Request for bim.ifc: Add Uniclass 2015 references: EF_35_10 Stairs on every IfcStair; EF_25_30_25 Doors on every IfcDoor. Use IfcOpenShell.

First a look at what the model holds.

```python
import ifcopenshell

model = ifcopenshell.open("bim.ifc")
print(model.schema)
print("classifications:", [c.Name for c in model.by_type("IfcClassification")])
for ifc_class in ("IfcDoor", "IfcRoof", "IfcStair", "IfcWall", "IfcWindow"):
    print(ifc_class, len(model.by_type(ifc_class)))
```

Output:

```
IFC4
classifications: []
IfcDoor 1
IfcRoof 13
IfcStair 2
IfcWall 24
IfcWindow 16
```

```python
import ifcopenshell
import ifcopenshell.api.classification

model = ifcopenshell.open("bim.ifc")

system = ifcopenshell.api.classification.add_classification(model, classification="Uniclass 2015")

codes = {
    "IfcStair": ("EF_35_10", "Stairs"),
    "IfcDoor": ("EF_25_30_25", "Doors"),
}
for ifc_class, (code, name) in codes.items():
    products = model.by_type(ifc_class)
    ifcopenshell.api.classification.add_reference(
        model, products=products, classification=system, identification=code, name=name
    )
    print(code, len(products))

model.write("bim_rev.ifc")
```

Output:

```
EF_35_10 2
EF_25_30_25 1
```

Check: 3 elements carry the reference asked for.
